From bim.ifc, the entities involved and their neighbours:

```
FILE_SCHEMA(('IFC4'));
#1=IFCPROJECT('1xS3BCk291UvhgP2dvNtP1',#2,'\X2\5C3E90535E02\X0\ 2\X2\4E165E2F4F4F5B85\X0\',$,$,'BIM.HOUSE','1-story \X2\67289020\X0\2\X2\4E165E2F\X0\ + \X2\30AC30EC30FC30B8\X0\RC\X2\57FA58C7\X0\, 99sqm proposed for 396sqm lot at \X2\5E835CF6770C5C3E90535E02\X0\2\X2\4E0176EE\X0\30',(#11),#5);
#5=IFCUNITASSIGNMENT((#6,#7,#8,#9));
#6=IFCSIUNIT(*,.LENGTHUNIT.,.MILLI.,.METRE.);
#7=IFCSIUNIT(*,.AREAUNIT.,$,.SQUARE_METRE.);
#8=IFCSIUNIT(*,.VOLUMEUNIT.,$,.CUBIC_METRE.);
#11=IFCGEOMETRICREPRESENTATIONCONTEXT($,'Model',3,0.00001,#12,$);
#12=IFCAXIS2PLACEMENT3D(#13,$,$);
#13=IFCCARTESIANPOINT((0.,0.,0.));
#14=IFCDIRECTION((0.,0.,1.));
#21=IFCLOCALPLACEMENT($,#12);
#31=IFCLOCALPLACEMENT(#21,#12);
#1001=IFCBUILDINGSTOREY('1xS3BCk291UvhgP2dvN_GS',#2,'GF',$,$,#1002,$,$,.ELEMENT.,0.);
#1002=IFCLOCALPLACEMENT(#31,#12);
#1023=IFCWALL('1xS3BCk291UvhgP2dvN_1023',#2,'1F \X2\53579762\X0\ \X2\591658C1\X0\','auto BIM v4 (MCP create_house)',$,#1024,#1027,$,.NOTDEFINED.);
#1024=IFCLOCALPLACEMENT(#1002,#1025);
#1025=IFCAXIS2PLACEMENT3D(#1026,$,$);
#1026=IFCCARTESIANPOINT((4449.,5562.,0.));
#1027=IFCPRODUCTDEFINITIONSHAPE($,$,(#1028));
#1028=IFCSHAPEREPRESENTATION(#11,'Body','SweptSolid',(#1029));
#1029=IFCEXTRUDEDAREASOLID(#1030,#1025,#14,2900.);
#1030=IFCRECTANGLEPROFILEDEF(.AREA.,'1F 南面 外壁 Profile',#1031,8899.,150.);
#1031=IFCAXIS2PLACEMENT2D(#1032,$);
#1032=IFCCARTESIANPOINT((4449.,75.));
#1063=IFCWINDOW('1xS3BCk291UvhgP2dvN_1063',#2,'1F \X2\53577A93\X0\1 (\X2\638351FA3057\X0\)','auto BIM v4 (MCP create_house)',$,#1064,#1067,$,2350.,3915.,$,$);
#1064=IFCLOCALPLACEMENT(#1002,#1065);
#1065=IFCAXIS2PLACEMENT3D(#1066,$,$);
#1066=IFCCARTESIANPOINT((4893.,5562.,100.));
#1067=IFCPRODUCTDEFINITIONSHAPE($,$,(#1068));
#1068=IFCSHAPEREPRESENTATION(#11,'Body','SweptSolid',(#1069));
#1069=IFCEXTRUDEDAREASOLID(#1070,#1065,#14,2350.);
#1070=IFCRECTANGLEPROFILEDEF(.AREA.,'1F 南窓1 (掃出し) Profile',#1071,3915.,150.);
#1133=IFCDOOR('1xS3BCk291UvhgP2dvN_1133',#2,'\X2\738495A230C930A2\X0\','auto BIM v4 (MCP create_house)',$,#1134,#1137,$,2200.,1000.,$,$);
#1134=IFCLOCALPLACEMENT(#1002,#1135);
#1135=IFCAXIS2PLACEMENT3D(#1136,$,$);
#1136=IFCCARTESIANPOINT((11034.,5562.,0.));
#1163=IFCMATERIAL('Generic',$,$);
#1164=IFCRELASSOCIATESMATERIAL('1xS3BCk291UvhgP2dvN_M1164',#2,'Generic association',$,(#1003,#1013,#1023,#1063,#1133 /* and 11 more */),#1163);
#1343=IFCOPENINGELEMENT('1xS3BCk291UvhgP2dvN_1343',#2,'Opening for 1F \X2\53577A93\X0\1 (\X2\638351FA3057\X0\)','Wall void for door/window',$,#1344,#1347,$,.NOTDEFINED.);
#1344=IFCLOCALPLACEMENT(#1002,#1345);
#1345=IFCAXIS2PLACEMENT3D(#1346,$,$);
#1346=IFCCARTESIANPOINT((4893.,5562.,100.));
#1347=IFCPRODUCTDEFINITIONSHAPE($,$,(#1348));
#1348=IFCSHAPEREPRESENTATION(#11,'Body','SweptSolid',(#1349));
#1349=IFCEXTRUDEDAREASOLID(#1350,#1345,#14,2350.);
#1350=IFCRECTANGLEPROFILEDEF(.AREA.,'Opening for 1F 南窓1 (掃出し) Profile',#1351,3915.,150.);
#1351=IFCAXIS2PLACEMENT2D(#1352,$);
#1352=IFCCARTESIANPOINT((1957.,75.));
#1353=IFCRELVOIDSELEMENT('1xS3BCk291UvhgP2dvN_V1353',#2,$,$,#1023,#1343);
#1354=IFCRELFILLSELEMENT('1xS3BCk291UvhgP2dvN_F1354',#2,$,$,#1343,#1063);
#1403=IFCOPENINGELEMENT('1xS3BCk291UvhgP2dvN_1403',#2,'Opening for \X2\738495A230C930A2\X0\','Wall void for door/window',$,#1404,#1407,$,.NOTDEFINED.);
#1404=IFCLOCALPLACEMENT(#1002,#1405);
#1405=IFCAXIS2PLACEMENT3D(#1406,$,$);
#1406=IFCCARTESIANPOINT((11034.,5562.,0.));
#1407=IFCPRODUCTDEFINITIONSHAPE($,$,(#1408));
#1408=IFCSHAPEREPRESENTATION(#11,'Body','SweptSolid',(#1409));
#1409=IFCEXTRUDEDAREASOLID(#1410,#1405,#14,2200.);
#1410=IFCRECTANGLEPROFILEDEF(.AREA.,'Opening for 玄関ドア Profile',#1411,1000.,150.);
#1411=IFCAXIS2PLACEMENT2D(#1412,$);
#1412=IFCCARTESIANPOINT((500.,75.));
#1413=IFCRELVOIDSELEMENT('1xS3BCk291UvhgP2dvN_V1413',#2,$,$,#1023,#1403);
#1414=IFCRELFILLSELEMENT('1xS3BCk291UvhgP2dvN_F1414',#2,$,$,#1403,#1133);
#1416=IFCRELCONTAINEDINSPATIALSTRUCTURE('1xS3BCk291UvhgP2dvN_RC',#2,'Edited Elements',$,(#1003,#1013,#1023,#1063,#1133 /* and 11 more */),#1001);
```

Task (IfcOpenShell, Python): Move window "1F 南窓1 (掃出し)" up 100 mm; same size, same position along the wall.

```python
import numpy as np
import ifcopenshell
import ifcopenshell.api.geometry
import ifcopenshell.util.placement
import ifcopenshell.util.unit

model = ifcopenshell.open("bim.ifc")
unit_scale = ifcopenshell.util.unit.calculate_unit_scale(model)

window = model.by_guid("1xS3BCk291UvhgP2dvN_1063")
opening = window.FillsVoids[0].RelatingOpeningElement
dz = 0.1 / unit_scale

shift = np.array([0.0, 0.0, dz])
# The window is not placed relative to its opening, so move both.
for product in (opening, window):
    matrix = ifcopenshell.util.placement.get_local_placement(product.ObjectPlacement)
    matrix[:3, 3] += shift
    ifcopenshell.api.geometry.edit_object_placement(model, product=product, matrix=matrix, is_si=False)

print(f"moved by {dz * unit_scale:+.3f} m")

model.write("bim_updated.ifc")
```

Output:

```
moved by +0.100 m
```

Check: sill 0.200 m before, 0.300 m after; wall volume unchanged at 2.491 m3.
